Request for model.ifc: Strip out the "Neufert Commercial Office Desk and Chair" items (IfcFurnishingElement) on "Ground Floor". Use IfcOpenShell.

First a look at what the model holds.

```python
import ifcopenshell
import ifcopenshell.util.element

model = ifcopenshell.open("model.ifc")
print(model.schema)
storey = next(s for s in model.by_type("IfcBuildingStorey") if s.Name == "Ground Floor")
furniture = [e for e in ifcopenshell.util.element.get_decomposition(storey) if e.is_a("IfcFurnishingElement")]
seen = {}
for e in furniture:
    element_type = ifcopenshell.util.element.get_type(e)
    name = element_type.Name if element_type not in (None, e) else None
    seen[name] = seen.get(name, 0) + 1
for name, count in sorted(seen.items(), key=str):
    print(count, "x", name)
```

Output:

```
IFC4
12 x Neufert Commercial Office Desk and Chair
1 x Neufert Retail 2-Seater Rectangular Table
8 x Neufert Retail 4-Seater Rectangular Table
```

```python
import ifcopenshell
import ifcopenshell.api.root
import ifcopenshell.util.element

model = ifcopenshell.open("model.ifc")

storey = next(s for s in model.by_type("IfcBuildingStorey") if s.Name == "Ground Floor")
furniture = [e for e in ifcopenshell.util.element.get_decomposition(storey) if e.is_a("IfcFurnishingElement")]
targets = [e for e in furniture if (t := ifcopenshell.util.element.get_type(e)) not in (None, e) and t.Name == "Neufert Commercial Office Desk and Chair"]

for e in targets:
    ifcopenshell.api.root.remove_product(model, product=e)
print(len(targets), "removed")

model.write("model_edited.ifc")
```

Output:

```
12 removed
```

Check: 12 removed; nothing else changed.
